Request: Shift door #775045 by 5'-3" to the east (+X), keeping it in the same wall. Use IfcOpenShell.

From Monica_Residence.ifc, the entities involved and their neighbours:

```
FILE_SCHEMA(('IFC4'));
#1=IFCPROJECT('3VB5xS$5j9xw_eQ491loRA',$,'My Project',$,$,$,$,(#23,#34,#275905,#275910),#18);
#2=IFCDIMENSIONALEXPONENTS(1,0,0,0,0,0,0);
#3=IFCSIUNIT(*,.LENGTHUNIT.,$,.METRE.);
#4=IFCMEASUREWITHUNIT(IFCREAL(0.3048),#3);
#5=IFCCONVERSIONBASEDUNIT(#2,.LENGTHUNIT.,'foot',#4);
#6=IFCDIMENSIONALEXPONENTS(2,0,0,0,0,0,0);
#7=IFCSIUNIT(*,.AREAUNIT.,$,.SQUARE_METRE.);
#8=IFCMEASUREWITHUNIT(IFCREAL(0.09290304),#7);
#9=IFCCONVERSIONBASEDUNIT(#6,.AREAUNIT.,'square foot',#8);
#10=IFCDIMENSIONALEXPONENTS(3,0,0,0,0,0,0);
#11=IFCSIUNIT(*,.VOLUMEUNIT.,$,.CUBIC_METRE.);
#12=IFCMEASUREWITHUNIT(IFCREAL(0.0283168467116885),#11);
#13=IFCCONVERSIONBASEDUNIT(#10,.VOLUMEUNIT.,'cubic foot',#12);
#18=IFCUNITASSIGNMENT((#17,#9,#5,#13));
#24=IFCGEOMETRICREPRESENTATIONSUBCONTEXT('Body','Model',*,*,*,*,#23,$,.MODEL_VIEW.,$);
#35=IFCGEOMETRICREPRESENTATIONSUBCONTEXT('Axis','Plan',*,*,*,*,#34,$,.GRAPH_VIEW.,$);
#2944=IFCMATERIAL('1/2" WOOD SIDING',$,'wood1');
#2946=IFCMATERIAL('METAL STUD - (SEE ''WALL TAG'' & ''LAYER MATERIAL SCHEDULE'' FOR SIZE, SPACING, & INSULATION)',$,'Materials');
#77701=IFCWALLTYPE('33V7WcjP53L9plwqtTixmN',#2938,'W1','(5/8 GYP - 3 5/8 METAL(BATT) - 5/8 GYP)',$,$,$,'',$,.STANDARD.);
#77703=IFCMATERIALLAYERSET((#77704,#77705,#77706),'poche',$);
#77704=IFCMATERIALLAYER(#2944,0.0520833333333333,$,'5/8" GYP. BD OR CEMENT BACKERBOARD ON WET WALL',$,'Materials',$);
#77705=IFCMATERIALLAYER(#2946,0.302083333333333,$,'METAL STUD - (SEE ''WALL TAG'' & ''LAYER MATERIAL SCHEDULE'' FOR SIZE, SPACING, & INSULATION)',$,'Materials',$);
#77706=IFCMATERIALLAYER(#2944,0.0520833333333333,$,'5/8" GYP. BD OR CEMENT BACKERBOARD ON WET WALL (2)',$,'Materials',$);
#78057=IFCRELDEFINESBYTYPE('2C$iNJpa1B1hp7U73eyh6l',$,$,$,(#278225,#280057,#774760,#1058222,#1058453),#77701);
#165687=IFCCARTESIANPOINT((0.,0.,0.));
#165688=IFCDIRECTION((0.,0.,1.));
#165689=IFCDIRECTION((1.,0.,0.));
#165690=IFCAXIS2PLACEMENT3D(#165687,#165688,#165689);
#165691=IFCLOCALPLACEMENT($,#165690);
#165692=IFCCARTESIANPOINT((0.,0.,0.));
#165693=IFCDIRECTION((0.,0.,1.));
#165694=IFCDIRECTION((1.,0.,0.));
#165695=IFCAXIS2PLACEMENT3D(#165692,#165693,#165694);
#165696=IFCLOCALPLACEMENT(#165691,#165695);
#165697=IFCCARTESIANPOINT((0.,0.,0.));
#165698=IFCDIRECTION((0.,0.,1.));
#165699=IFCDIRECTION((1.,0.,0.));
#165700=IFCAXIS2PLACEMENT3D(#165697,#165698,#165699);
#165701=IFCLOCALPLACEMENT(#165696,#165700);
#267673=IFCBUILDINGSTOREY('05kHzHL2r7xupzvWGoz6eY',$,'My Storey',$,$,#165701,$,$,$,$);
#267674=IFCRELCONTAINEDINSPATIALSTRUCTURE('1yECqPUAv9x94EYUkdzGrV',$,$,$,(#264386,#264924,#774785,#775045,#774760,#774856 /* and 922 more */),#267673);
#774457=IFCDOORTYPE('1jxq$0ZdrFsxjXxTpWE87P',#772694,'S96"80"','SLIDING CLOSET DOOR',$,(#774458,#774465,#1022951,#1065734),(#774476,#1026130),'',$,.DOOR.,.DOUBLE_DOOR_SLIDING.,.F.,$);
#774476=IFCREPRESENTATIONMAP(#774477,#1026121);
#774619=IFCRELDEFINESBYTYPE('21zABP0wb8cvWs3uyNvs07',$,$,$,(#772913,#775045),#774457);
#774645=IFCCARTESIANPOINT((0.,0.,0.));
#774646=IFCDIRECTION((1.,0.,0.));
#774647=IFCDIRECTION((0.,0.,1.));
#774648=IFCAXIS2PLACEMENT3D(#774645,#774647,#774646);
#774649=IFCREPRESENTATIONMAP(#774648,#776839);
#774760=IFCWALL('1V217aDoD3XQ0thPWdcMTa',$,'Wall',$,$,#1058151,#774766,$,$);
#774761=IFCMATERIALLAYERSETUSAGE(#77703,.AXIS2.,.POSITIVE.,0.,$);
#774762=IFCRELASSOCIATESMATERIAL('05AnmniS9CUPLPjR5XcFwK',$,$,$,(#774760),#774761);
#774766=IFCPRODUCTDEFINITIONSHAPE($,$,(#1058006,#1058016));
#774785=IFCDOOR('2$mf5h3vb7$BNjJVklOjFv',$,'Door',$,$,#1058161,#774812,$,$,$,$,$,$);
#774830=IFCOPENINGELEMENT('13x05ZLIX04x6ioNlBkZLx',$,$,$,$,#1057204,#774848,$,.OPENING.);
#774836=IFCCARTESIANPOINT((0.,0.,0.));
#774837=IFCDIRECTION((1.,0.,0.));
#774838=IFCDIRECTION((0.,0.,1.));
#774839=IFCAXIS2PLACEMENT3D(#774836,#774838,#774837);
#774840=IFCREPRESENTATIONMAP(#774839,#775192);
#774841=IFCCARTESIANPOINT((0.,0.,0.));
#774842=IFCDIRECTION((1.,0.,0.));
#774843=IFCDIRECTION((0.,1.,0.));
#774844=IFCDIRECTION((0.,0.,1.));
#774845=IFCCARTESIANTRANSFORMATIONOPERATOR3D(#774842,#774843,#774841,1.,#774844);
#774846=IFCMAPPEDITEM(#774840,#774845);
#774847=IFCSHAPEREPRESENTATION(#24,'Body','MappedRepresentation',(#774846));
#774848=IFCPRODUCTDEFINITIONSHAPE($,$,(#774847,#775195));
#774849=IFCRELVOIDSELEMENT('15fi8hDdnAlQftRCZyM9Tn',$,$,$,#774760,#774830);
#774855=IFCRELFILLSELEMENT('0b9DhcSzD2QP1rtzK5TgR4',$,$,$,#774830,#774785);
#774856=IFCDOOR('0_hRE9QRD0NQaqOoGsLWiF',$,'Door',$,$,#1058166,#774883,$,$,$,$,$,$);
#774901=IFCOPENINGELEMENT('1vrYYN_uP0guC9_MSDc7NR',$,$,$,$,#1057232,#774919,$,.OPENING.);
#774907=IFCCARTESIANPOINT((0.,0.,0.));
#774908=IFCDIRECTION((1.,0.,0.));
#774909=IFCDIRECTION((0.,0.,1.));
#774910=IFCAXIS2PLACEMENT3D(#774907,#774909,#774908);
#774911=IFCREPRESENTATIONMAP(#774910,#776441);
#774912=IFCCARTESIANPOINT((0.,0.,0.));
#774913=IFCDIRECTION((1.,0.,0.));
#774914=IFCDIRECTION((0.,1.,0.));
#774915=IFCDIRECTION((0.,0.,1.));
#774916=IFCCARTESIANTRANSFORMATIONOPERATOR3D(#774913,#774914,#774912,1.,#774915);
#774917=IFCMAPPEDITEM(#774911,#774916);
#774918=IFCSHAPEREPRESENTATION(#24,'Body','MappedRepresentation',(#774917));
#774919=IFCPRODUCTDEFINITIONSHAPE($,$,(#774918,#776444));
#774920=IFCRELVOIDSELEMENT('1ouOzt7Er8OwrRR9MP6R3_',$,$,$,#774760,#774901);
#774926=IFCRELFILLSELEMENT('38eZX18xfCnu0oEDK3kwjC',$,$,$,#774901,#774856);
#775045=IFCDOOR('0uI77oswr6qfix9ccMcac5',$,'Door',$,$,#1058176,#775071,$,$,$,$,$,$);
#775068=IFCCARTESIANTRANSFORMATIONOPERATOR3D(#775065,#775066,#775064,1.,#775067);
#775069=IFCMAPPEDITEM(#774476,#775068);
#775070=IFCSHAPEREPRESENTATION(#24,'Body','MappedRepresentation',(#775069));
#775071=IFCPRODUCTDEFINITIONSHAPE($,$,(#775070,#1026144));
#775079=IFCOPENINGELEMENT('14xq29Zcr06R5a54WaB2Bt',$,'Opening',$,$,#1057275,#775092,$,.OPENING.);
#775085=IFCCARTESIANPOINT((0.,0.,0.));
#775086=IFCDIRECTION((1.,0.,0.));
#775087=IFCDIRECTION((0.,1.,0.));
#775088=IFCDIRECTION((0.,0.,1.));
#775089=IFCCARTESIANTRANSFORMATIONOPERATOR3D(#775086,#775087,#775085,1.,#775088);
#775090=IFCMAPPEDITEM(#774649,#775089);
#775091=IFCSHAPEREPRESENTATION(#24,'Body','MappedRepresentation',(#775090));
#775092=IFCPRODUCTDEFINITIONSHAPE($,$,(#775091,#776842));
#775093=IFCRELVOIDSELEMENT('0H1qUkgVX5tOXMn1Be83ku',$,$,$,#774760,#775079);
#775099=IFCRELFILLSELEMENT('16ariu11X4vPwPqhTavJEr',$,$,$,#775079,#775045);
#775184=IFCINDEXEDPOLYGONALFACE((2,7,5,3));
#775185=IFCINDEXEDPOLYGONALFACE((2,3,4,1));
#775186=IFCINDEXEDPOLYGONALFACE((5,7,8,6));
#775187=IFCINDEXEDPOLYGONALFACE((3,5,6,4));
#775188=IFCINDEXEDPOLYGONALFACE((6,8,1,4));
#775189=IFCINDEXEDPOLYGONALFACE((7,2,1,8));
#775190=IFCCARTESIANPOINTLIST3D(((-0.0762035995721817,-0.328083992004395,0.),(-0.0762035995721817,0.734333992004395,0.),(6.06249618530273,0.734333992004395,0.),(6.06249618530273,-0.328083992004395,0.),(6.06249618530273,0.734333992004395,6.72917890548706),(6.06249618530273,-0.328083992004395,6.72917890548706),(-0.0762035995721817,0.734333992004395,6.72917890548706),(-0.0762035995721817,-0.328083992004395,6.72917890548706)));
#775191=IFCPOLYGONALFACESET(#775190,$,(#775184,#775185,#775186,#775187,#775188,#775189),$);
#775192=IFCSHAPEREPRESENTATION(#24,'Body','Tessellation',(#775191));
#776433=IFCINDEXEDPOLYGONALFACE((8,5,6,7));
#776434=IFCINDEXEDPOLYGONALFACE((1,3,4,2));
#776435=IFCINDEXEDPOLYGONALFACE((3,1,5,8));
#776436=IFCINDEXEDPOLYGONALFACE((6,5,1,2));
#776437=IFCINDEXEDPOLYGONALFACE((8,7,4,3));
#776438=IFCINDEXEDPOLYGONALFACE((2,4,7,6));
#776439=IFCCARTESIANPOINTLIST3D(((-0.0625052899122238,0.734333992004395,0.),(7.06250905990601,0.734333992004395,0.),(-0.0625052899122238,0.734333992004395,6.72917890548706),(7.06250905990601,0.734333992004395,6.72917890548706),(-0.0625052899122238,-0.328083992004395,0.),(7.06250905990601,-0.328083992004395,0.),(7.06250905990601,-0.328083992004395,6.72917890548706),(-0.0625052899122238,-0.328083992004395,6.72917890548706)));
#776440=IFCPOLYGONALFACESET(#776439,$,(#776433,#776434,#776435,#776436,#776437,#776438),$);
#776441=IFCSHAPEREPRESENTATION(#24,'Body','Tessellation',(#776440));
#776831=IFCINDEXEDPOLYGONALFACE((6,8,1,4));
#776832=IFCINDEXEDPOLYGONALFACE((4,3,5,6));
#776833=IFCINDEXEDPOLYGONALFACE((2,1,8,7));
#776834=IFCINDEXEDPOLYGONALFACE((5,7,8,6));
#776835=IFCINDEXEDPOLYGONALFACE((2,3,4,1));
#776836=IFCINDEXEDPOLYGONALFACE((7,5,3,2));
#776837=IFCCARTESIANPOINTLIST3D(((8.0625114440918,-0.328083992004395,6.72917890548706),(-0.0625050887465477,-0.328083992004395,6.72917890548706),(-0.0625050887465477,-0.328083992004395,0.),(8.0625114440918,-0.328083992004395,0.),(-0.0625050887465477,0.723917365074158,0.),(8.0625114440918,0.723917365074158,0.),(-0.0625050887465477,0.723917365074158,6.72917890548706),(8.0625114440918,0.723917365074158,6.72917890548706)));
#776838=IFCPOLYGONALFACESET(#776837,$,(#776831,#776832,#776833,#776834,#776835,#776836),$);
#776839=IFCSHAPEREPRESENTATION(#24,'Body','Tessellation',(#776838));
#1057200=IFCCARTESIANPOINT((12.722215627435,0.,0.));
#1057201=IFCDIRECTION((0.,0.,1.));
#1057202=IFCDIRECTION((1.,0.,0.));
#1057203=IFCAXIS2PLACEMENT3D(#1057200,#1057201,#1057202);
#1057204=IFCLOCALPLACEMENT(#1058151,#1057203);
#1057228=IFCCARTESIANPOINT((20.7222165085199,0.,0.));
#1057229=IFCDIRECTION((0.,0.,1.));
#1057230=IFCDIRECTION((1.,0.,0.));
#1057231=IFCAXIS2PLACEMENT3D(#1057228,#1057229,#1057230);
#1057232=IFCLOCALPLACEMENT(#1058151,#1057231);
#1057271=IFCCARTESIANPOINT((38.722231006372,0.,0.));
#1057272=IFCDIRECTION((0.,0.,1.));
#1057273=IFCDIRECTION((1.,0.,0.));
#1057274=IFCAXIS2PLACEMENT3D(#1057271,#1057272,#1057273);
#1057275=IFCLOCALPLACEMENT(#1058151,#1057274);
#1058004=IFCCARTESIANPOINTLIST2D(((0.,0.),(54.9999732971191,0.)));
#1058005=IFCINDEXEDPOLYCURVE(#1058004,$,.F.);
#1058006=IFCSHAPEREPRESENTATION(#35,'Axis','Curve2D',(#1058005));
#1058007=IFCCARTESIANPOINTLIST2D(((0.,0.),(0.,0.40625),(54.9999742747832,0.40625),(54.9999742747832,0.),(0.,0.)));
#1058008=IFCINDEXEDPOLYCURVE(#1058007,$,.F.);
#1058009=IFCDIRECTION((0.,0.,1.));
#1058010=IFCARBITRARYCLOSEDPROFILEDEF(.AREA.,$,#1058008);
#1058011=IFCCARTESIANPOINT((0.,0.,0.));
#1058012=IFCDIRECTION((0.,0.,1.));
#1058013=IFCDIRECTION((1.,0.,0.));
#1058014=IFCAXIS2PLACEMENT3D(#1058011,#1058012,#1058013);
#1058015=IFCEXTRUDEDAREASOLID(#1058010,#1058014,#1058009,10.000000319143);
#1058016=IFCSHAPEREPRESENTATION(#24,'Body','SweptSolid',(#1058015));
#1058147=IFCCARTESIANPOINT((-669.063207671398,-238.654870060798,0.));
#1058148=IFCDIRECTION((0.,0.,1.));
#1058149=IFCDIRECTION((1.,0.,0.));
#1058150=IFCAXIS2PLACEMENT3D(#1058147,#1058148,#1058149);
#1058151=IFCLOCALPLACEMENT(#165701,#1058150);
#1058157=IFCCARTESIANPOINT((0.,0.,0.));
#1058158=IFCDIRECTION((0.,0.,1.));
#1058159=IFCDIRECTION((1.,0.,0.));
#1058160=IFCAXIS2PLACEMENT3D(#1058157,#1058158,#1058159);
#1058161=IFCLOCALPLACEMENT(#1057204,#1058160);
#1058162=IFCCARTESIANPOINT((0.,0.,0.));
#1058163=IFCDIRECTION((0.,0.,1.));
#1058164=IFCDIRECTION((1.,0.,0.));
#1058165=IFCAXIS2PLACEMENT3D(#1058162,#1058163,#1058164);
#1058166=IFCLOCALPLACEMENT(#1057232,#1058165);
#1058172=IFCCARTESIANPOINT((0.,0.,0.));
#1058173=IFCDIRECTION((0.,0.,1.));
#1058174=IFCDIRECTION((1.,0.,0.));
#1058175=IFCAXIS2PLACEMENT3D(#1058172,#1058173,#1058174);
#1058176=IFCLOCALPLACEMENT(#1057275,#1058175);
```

```python
import ifcopenshell
import ifcopenshell.api.geometry
import ifcopenshell.util.placement
import ifcopenshell.util.unit

model = ifcopenshell.open("Monica_Residence.ifc")
unit_scale = ifcopenshell.util.unit.calculate_unit_scale(model)

door = model.by_id(775045)
opening = door.FillsVoids[0].RelatingOpeningElement
wall = opening.VoidsElements[0].RelatingBuildingElement

wall_matrix = ifcopenshell.util.placement.get_local_placement(wall.ObjectPlacement)
shift = wall_matrix[:3, 0] * 63 * 0.0254 / unit_scale
before = ifcopenshell.util.placement.get_local_placement(door.ObjectPlacement)[:3, 3].copy()

# The door is placed relative to its opening, so it follows when the opening moves.
matrix = ifcopenshell.util.placement.get_local_placement(opening.ObjectPlacement)
matrix[:3, 3] += shift
ifcopenshell.api.geometry.edit_object_placement(
    model, product=opening, matrix=matrix, is_si=False, should_transform_children=True
)

after = ifcopenshell.util.placement.get_local_placement(door.ObjectPlacement)[:3, 3]
print("door moved by", (after - before).round(3) + 0.0)

model.write("Monica_Residence_edited.ifc")
```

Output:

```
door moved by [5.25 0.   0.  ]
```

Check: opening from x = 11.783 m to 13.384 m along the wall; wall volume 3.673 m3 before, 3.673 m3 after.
